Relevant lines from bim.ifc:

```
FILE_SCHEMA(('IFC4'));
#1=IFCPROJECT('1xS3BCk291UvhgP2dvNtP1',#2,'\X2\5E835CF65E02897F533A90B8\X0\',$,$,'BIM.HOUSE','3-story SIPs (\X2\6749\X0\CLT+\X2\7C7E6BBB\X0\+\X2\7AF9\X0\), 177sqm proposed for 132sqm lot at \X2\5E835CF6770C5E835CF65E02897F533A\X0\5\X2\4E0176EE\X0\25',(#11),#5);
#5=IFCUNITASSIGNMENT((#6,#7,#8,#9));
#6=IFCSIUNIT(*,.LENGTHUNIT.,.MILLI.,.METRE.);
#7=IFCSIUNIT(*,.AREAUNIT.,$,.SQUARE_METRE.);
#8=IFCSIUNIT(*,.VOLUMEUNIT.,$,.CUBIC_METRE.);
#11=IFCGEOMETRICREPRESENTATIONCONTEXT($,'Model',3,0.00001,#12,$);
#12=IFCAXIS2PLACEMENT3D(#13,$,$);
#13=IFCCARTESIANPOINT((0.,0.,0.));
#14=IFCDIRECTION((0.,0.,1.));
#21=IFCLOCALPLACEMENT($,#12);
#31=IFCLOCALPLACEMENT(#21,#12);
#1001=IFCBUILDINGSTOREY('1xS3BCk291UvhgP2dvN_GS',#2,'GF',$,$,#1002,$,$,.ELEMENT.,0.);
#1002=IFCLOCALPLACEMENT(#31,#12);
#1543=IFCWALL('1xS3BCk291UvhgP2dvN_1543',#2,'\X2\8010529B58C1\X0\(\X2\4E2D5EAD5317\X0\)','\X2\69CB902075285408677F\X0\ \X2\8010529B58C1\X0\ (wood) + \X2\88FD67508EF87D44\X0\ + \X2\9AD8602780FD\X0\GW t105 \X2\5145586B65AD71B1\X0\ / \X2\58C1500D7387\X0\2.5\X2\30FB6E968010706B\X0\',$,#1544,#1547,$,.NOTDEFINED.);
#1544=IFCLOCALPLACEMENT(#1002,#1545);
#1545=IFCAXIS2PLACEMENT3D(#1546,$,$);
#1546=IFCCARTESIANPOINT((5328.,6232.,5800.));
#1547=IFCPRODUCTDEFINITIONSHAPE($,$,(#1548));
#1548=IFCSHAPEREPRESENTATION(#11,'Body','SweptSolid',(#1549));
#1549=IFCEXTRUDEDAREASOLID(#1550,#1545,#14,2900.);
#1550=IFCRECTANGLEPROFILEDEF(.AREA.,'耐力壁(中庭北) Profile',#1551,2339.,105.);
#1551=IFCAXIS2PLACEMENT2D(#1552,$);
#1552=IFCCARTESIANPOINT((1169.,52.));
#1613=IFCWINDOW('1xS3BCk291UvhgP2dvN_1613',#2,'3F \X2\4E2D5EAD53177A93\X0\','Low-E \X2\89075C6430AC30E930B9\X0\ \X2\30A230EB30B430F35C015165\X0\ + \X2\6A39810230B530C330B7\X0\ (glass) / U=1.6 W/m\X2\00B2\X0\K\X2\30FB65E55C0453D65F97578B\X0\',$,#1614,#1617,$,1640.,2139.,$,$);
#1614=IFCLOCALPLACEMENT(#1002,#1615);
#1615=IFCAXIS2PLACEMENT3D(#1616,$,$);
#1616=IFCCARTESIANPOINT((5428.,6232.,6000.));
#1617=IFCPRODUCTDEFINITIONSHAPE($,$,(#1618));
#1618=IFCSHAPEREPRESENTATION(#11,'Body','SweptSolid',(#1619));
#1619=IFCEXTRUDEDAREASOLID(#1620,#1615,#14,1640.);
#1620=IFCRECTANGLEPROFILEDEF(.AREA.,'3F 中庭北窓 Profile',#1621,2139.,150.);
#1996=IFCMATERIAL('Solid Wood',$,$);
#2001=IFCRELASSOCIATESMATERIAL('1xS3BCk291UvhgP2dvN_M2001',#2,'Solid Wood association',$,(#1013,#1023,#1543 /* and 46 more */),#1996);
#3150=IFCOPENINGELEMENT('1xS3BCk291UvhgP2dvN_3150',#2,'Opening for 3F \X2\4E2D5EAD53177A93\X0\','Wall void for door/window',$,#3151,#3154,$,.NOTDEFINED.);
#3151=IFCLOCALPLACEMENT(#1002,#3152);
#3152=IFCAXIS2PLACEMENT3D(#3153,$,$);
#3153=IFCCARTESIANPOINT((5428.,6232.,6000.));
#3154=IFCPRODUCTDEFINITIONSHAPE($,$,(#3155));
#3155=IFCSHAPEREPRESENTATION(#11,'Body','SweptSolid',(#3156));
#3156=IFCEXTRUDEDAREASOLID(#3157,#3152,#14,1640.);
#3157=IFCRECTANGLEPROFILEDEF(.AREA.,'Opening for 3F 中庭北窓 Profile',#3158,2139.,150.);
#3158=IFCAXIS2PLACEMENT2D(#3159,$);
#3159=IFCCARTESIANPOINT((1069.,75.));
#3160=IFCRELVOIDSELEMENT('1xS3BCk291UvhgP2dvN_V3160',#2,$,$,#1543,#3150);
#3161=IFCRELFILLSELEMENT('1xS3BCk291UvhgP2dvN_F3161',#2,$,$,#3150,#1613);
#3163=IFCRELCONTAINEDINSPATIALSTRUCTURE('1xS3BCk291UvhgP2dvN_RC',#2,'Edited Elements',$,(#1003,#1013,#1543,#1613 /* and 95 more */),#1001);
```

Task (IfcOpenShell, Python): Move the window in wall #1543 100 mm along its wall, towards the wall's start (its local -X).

```python
import ifcopenshell
import ifcopenshell.api.geometry
import ifcopenshell.util.placement

model = ifcopenshell.open("bim.ifc")

window = model.by_guid("1xS3BCk291UvhgP2dvN_1613")
opening = window.FillsVoids[0].RelatingOpeningElement
wall = opening.VoidsElements[0].RelatingBuildingElement

wall_matrix = ifcopenshell.util.placement.get_local_placement(wall.ObjectPlacement)
shift = wall_matrix[:3, 0] * -100.0
before = ifcopenshell.util.placement.get_local_placement(window.ObjectPlacement)[:3, 3].copy()

# The window is not placed relative to its opening, so move both.
for product in (opening, window):
    matrix = ifcopenshell.util.placement.get_local_placement(product.ObjectPlacement)
    matrix[:3, 3] += shift
    ifcopenshell.api.geometry.edit_object_placement(model, product=product, matrix=matrix, is_si=False)

after = ifcopenshell.util.placement.get_local_placement(window.ObjectPlacement)[:3, 3]
print("window moved by", (after - before).round(3) + 0.0)

model.write("bim_updated.ifc")
```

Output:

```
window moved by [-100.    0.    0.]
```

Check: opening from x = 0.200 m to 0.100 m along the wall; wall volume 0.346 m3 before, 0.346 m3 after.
